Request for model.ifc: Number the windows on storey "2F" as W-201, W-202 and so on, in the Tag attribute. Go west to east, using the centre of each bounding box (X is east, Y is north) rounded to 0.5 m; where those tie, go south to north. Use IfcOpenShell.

First a look at what the model holds.

```python
import ifcopenshell
import ifcopenshell.util.element
import ifcopenshell.util.placement

model = ifcopenshell.open("model.ifc")
print(model.schema)
storey = next(s for s in model.by_type("IfcBuildingStorey") if s.Name == "2F")
windows = [e for e in ifcopenshell.util.element.get_decomposition(storey) if e.is_a("IfcWindow")]
for e in sorted(windows, key=lambda e: e.id()):
    origin = ifcopenshell.util.placement.get_local_placement(e.ObjectPlacement)[:3, 3]
    print(e.id(), e.Tag, e.Name, origin.round(2) + 0.0, sep=" | ")
```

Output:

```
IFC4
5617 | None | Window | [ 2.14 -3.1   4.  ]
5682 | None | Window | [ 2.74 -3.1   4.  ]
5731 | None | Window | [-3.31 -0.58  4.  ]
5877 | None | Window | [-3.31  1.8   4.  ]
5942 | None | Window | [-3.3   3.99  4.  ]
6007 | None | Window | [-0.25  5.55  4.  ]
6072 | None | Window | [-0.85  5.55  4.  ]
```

```python
import ifcopenshell
import ifcopenshell.geom
import ifcopenshell.util.element
import ifcopenshell.util.shape

model = ifcopenshell.open("model.ifc")
settings = ifcopenshell.geom.settings()
settings.set("use-world-coords", True)


def centre(element):
    shape = ifcopenshell.geom.create_shape(settings, element)
    return ifcopenshell.util.shape.get_bbox_centroid(shape.geometry)


storey = next(s for s in model.by_type("IfcBuildingStorey") if s.Name == "2F")
windows = [e for e in ifcopenshell.util.element.get_decomposition(storey) if e.is_a("IfcWindow")]

# Insertion points can sit at a corner or the storey origin, so sort by the geometry (in metres).
centres = {e: centre(e) for e in windows}
windows.sort(key=lambda e: (round(centres[e][0] / 0.5), centres[e][1]))

for i, e in enumerate(windows, start=1):
    number = f"W-2{i:02d}"
    e.Tag = number
    print(e.id(), number)

model.write("model-out.ifc")
```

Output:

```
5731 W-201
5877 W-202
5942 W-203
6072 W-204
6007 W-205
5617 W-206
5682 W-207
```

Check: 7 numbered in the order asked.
